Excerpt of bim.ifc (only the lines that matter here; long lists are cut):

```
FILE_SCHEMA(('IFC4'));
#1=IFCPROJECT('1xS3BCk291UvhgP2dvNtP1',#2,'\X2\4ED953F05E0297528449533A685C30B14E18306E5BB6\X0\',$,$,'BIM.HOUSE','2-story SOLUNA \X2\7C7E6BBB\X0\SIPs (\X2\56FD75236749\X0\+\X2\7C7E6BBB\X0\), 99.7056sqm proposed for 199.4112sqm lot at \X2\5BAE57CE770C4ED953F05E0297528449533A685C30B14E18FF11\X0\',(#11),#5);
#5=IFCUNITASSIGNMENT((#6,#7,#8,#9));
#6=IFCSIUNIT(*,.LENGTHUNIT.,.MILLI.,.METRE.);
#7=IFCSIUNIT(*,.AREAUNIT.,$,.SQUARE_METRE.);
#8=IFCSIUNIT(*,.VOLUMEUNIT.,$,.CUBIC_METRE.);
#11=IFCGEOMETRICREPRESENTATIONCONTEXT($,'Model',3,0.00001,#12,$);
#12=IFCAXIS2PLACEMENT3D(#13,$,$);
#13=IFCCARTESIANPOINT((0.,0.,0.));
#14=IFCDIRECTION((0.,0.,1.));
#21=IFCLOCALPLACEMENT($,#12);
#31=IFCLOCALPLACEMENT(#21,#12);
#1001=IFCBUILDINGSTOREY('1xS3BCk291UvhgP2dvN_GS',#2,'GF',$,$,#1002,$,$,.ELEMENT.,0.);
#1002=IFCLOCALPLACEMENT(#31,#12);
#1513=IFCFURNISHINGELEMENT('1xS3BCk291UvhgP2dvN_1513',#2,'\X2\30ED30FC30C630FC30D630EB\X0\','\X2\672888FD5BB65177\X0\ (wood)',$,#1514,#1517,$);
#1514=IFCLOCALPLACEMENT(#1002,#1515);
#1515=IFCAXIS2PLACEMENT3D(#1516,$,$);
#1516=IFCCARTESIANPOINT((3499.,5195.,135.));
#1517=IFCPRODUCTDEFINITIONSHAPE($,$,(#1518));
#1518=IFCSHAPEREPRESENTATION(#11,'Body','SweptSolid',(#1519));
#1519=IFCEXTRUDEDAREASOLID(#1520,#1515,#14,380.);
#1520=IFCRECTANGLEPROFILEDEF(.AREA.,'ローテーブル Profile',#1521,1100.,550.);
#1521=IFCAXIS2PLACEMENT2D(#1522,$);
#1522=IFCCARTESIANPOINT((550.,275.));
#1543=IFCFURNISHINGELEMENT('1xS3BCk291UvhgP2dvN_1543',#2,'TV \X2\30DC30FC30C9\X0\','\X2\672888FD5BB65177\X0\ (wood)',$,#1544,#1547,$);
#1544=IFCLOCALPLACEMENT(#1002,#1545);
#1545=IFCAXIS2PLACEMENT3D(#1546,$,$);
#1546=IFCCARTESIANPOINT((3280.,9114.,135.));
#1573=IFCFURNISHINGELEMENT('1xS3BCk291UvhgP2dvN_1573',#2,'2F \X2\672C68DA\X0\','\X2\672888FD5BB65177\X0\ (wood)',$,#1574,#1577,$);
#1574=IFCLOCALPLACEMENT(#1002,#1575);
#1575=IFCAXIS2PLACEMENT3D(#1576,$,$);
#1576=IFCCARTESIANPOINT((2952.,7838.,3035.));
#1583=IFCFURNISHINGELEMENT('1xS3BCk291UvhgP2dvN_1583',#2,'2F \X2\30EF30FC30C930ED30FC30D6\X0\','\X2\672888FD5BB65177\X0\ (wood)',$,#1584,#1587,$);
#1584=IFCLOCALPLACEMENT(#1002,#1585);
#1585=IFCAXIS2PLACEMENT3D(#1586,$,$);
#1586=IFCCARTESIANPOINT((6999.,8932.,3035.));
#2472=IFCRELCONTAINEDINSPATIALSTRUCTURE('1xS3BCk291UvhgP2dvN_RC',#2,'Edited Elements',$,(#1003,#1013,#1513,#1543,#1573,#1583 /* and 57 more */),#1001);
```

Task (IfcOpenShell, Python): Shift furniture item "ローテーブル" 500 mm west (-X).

```python
import ifcopenshell
import ifcopenshell.api.geometry
import ifcopenshell.util.placement

model = ifcopenshell.open("bim.ifc")

item = model.by_guid("1xS3BCk291UvhgP2dvN_1513")
matrix = ifcopenshell.util.placement.get_local_placement(item.ObjectPlacement)
matrix[0, 3] -= 500.0
ifcopenshell.api.geometry.edit_object_placement(model, product=item, matrix=matrix, is_si=False)

print(ifcopenshell.util.placement.get_local_placement(item.ObjectPlacement).round(3) + 0.0)

model.write("bim_v2.ifc")
```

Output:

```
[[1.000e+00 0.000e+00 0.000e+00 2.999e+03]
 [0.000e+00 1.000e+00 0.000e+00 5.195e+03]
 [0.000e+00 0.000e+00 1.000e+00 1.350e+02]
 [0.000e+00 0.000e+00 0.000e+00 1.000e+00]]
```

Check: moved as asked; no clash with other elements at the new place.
